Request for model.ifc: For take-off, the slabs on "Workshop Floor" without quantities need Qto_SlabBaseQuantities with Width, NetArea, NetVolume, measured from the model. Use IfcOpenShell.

First a look at what the model holds.

```python
import ifcopenshell
import ifcopenshell.util.element
import ifcopenshell.util.unit

model = ifcopenshell.open("model.ifc")
print(model.schema)
for unit_type in ("LENGTHUNIT", "AREAUNIT", "VOLUMEUNIT"):
    print(unit_type, ifcopenshell.util.unit.calculate_unit_scale(model, unit_type))
storey = next(s for s in model.by_type("IfcBuildingStorey") if s.Name == "Workshop Floor")
slabs = [e for e in ifcopenshell.util.element.get_decomposition(storey) if e.is_a("IfcSlab")]
for e in sorted(slabs, key=lambda e: e.id()):
    print(e.id(), e.is_a(), e.Name, list(ifcopenshell.util.element.get_psets(e, qtos_only=True)), sep=" | ")
```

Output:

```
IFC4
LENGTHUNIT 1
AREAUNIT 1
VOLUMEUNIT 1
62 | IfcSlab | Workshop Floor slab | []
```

```python
import ifcopenshell
import ifcopenshell.api.pset
import ifcopenshell.geom
import ifcopenshell.util.element
import ifcopenshell.util.shape
import ifcopenshell.util.unit

model = ifcopenshell.open("model.ifc")
unit_scale = ifcopenshell.util.unit.calculate_unit_scale(model)
area_scale = ifcopenshell.util.unit.calculate_unit_scale(model, "AREAUNIT")
volume_scale = ifcopenshell.util.unit.calculate_unit_scale(model, "VOLUMEUNIT")
settings = ifcopenshell.geom.settings()

storey = next(s for s in model.by_type("IfcBuildingStorey") if s.Name == "Workshop Floor")
slabs = [e for e in ifcopenshell.util.element.get_decomposition(storey) if e.is_a("IfcSlab")]

for e in sorted(slabs, key=lambda e: e.id()):
    if ifcopenshell.util.element.get_psets(e, qtos_only=True, should_inherit=False):
        continue
    # Geometry comes back in metres, in the element's own axes.
    shape = ifcopenshell.geom.create_shape(settings, e)
    values = {
        "Width": ifcopenshell.util.shape.get_z(shape.geometry) / unit_scale,
        "NetArea": ifcopenshell.util.shape.get_footprint_area(shape.geometry) / area_scale,
        "NetVolume": ifcopenshell.util.shape.get_volume(shape.geometry) / volume_scale,
    }
    qto = ifcopenshell.api.pset.add_qto(model, product=e, name="Qto_SlabBaseQuantities")
    ifcopenshell.api.pset.edit_qto(model, qto=qto, properties=values)
    print(e.id(), {k: round(v, 3) for k, v in values.items()})

model.write("model_v2.ifc")
```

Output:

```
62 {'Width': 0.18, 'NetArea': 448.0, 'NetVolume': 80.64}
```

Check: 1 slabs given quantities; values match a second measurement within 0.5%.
